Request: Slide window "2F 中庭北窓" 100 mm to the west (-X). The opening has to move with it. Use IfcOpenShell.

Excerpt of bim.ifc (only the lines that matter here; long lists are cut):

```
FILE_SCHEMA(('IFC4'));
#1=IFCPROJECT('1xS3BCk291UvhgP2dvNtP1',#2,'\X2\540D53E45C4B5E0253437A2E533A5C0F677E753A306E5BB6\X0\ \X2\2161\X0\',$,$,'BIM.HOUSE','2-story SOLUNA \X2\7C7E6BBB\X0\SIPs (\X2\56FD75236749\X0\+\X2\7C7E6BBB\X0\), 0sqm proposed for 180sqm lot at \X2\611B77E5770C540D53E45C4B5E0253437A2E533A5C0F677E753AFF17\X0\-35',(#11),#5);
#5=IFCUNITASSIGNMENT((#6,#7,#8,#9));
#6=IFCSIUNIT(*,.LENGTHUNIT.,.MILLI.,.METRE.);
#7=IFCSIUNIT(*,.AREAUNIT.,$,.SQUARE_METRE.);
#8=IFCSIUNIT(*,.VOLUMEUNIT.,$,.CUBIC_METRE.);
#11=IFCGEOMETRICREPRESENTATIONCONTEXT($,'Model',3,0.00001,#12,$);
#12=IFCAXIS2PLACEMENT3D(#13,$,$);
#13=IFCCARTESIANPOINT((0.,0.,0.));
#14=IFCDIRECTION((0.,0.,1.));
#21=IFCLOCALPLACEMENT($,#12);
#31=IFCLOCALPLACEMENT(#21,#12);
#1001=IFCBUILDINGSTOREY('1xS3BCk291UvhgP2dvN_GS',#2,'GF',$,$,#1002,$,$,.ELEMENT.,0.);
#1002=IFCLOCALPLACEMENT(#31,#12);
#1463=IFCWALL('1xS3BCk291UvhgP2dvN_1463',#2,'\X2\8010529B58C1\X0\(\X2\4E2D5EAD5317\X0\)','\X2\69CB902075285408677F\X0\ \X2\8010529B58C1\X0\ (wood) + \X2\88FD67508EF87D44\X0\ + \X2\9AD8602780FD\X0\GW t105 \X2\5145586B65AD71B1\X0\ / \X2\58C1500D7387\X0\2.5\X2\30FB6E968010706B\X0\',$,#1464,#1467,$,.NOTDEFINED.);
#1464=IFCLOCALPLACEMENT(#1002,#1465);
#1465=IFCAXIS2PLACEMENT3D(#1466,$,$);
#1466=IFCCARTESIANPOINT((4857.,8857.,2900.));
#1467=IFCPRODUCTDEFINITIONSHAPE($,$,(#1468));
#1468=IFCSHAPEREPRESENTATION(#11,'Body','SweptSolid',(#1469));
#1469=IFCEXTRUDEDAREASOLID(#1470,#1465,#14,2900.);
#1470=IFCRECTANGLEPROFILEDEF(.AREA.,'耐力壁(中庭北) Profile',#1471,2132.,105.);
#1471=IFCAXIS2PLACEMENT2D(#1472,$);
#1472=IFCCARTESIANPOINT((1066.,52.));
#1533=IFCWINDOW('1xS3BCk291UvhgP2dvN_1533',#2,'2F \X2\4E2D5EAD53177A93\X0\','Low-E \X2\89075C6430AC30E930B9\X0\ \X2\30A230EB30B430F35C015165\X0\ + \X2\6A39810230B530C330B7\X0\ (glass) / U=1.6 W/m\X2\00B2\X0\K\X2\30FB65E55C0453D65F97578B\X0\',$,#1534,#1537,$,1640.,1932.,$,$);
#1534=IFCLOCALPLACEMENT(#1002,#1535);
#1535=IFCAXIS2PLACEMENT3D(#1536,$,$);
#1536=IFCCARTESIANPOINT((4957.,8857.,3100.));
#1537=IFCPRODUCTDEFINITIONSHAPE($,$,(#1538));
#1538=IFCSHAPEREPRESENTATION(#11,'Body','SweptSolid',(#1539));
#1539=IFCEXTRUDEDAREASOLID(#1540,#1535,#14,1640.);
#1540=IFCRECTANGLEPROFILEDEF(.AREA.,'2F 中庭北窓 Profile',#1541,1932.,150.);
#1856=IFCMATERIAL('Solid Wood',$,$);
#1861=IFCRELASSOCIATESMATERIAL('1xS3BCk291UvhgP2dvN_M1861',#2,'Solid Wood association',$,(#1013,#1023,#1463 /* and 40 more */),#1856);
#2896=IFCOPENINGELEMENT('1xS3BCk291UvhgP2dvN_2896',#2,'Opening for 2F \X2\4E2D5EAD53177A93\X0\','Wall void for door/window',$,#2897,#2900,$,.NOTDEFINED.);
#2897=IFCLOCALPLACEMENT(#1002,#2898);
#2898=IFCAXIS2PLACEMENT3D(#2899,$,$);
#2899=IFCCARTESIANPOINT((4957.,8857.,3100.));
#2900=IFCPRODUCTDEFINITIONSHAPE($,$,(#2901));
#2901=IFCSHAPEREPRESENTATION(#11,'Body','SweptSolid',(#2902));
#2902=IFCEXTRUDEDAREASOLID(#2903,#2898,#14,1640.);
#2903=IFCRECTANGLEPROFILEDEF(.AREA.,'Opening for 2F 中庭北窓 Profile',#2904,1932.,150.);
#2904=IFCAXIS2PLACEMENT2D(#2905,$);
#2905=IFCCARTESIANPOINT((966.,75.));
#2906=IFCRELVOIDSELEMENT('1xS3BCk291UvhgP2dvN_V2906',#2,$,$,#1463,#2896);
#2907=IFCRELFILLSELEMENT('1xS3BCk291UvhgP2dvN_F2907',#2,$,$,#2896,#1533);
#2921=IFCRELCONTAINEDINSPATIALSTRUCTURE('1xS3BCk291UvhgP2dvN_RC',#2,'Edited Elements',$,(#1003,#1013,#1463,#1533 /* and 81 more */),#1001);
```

```python
import ifcopenshell
import ifcopenshell.api.geometry
import ifcopenshell.util.placement

model = ifcopenshell.open("bim.ifc")

window = model.by_id(1533)
opening = window.FillsVoids[0].RelatingOpeningElement
wall = opening.VoidsElements[0].RelatingBuildingElement

wall_matrix = ifcopenshell.util.placement.get_local_placement(wall.ObjectPlacement)
shift = wall_matrix[:3, 0] * -100.0
before = ifcopenshell.util.placement.get_local_placement(window.ObjectPlacement)[:3, 3].copy()

# The window is not placed relative to its opening, so move both.
for product in (opening, window):
    matrix = ifcopenshell.util.placement.get_local_placement(product.ObjectPlacement)
    matrix[:3, 3] += shift
    ifcopenshell.api.geometry.edit_object_placement(model, product=product, matrix=matrix, is_si=False)

after = ifcopenshell.util.placement.get_local_placement(window.ObjectPlacement)[:3, 3]
print("window moved by", (after - before).round(3) + 0.0)

model.write("bim_rev.ifc")
```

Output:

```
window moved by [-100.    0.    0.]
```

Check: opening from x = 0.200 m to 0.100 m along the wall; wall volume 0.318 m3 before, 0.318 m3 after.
